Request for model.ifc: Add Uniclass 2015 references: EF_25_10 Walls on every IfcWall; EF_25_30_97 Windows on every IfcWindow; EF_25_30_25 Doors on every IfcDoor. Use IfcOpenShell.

First a look at what the model holds.

```python
import ifcopenshell

model = ifcopenshell.open("model.ifc")
print(model.schema)
print("classifications:", [c.Name for c in model.by_type("IfcClassification")])
for ifc_class in ("IfcDoor", "IfcRoof", "IfcStair", "IfcWall", "IfcWindow"):
    print(ifc_class, len(model.by_type(ifc_class)))
```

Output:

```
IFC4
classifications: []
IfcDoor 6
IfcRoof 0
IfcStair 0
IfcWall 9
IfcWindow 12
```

```python
import ifcopenshell
import ifcopenshell.api.classification

model = ifcopenshell.open("model.ifc")

system = ifcopenshell.api.classification.add_classification(model, classification="Uniclass 2015")

codes = {
    "IfcWall": ("EF_25_10", "Walls"),
    "IfcWindow": ("EF_25_30_97", "Windows"),
    "IfcDoor": ("EF_25_30_25", "Doors"),
}
for ifc_class, (code, name) in codes.items():
    products = model.by_type(ifc_class)
    ifcopenshell.api.classification.add_reference(
        model, products=products, classification=system, identification=code, name=name
    )
    print(code, len(products))

model.write("model-out.ifc")
```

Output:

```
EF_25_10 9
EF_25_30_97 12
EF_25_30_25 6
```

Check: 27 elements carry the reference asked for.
